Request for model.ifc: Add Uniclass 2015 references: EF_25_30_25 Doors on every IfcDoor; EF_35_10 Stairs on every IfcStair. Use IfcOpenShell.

First a look at what the model holds.

```python
import ifcopenshell

model = ifcopenshell.open("model.ifc")
print(model.schema)
print("classifications:", [c.Name for c in model.by_type("IfcClassification")])
for ifc_class in ("IfcDoor", "IfcRoof", "IfcStair", "IfcWall", "IfcWindow"):
    print(ifc_class, len(model.by_type(ifc_class)))
```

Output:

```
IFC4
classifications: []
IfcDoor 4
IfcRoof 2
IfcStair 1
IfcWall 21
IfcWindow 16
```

```python
import ifcopenshell
import ifcopenshell.api.classification

model = ifcopenshell.open("model.ifc")

system = ifcopenshell.api.classification.add_classification(model, classification="Uniclass 2015")

codes = {
    "IfcDoor": ("EF_25_30_25", "Doors"),
    "IfcStair": ("EF_35_10", "Stairs"),
}
for ifc_class, (code, name) in codes.items():
    products = model.by_type(ifc_class)
    ifcopenshell.api.classification.add_reference(
        model, products=products, classification=system, identification=code, name=name
    )
    print(code, len(products))

model.write("model-out.ifc")
```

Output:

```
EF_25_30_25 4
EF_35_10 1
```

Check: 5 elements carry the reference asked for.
